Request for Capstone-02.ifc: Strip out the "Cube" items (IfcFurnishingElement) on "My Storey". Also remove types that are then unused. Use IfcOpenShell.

First a look at what the model holds.

```python
import ifcopenshell
import ifcopenshell.util.element

model = ifcopenshell.open("Capstone-02.ifc")
print(model.schema)
storey = next(s for s in model.by_type("IfcBuildingStorey") if s.Name == "My Storey")
furniture = [e for e in ifcopenshell.util.element.get_decomposition(storey) if e.is_a("IfcFurnishingElement")]
seen = {}
for e in furniture:
    element_type = ifcopenshell.util.element.get_type(e)
    name = element_type.Name if element_type not in (None, e) else None
    seen[name] = seen.get(name, 0) + 1
for name, count in sorted(seen.items(), key=str):
    print(count, "x", name)
```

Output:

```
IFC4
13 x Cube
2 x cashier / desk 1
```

```python
import ifcopenshell
import ifcopenshell.api.root
import ifcopenshell.util.element

model = ifcopenshell.open("Capstone-02.ifc")

storey = next(s for s in model.by_type("IfcBuildingStorey") if s.Name == "My Storey")
furniture = [e for e in ifcopenshell.util.element.get_decomposition(storey) if e.is_a("IfcFurnishingElement")]
targets = [e for e in furniture if (t := ifcopenshell.util.element.get_type(e)) not in (None, e) and t.Name == "Cube"]
types = {ifcopenshell.util.element.get_type(e) for e in targets} - {None, *targets}

for e in targets:
    ifcopenshell.api.root.remove_product(model, product=e)
print(len(targets), "removed")

unused = [t for t in types if not ifcopenshell.util.element.get_types(t)]
for t in unused:
    ifcopenshell.api.root.remove_product(model, product=t)
print(len(unused), "unused types removed")

model.write("Capstone-02-out.ifc")
```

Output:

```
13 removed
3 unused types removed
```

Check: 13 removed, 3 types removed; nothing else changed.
